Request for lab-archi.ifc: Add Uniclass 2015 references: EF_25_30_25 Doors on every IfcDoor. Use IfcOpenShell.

First a look at what the model holds.

```python
import ifcopenshell

model = ifcopenshell.open("lab-archi.ifc")
print(model.schema)
print("classifications:", [c.Name for c in model.by_type("IfcClassification")])
for ifc_class in ("IfcDoor", "IfcRoof", "IfcStair", "IfcWall", "IfcWindow"):
    print(ifc_class, len(model.by_type(ifc_class)))
```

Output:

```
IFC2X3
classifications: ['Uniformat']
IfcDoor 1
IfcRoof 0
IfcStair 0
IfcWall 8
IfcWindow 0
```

```python
import ifcopenshell
import ifcopenshell.api.classification

model = ifcopenshell.open("lab-archi.ifc")

# IFC2X3 requires Source and Edition and has no link from the project to the system.
system = model.create_entity("IfcClassification", Source="NBS", Edition="2015", Name="Uniclass 2015")

codes = {
    "IfcDoor": ("EF_25_30_25", "Doors"),
}
for ifc_class, (code, name) in codes.items():
    products = model.by_type(ifc_class)
    ifcopenshell.api.classification.add_reference(
        model, products=products, classification=system, identification=code, name=name
    )
    print(code, len(products))

model.write("lab-archi_updated.ifc")
```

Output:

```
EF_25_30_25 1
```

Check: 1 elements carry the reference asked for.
